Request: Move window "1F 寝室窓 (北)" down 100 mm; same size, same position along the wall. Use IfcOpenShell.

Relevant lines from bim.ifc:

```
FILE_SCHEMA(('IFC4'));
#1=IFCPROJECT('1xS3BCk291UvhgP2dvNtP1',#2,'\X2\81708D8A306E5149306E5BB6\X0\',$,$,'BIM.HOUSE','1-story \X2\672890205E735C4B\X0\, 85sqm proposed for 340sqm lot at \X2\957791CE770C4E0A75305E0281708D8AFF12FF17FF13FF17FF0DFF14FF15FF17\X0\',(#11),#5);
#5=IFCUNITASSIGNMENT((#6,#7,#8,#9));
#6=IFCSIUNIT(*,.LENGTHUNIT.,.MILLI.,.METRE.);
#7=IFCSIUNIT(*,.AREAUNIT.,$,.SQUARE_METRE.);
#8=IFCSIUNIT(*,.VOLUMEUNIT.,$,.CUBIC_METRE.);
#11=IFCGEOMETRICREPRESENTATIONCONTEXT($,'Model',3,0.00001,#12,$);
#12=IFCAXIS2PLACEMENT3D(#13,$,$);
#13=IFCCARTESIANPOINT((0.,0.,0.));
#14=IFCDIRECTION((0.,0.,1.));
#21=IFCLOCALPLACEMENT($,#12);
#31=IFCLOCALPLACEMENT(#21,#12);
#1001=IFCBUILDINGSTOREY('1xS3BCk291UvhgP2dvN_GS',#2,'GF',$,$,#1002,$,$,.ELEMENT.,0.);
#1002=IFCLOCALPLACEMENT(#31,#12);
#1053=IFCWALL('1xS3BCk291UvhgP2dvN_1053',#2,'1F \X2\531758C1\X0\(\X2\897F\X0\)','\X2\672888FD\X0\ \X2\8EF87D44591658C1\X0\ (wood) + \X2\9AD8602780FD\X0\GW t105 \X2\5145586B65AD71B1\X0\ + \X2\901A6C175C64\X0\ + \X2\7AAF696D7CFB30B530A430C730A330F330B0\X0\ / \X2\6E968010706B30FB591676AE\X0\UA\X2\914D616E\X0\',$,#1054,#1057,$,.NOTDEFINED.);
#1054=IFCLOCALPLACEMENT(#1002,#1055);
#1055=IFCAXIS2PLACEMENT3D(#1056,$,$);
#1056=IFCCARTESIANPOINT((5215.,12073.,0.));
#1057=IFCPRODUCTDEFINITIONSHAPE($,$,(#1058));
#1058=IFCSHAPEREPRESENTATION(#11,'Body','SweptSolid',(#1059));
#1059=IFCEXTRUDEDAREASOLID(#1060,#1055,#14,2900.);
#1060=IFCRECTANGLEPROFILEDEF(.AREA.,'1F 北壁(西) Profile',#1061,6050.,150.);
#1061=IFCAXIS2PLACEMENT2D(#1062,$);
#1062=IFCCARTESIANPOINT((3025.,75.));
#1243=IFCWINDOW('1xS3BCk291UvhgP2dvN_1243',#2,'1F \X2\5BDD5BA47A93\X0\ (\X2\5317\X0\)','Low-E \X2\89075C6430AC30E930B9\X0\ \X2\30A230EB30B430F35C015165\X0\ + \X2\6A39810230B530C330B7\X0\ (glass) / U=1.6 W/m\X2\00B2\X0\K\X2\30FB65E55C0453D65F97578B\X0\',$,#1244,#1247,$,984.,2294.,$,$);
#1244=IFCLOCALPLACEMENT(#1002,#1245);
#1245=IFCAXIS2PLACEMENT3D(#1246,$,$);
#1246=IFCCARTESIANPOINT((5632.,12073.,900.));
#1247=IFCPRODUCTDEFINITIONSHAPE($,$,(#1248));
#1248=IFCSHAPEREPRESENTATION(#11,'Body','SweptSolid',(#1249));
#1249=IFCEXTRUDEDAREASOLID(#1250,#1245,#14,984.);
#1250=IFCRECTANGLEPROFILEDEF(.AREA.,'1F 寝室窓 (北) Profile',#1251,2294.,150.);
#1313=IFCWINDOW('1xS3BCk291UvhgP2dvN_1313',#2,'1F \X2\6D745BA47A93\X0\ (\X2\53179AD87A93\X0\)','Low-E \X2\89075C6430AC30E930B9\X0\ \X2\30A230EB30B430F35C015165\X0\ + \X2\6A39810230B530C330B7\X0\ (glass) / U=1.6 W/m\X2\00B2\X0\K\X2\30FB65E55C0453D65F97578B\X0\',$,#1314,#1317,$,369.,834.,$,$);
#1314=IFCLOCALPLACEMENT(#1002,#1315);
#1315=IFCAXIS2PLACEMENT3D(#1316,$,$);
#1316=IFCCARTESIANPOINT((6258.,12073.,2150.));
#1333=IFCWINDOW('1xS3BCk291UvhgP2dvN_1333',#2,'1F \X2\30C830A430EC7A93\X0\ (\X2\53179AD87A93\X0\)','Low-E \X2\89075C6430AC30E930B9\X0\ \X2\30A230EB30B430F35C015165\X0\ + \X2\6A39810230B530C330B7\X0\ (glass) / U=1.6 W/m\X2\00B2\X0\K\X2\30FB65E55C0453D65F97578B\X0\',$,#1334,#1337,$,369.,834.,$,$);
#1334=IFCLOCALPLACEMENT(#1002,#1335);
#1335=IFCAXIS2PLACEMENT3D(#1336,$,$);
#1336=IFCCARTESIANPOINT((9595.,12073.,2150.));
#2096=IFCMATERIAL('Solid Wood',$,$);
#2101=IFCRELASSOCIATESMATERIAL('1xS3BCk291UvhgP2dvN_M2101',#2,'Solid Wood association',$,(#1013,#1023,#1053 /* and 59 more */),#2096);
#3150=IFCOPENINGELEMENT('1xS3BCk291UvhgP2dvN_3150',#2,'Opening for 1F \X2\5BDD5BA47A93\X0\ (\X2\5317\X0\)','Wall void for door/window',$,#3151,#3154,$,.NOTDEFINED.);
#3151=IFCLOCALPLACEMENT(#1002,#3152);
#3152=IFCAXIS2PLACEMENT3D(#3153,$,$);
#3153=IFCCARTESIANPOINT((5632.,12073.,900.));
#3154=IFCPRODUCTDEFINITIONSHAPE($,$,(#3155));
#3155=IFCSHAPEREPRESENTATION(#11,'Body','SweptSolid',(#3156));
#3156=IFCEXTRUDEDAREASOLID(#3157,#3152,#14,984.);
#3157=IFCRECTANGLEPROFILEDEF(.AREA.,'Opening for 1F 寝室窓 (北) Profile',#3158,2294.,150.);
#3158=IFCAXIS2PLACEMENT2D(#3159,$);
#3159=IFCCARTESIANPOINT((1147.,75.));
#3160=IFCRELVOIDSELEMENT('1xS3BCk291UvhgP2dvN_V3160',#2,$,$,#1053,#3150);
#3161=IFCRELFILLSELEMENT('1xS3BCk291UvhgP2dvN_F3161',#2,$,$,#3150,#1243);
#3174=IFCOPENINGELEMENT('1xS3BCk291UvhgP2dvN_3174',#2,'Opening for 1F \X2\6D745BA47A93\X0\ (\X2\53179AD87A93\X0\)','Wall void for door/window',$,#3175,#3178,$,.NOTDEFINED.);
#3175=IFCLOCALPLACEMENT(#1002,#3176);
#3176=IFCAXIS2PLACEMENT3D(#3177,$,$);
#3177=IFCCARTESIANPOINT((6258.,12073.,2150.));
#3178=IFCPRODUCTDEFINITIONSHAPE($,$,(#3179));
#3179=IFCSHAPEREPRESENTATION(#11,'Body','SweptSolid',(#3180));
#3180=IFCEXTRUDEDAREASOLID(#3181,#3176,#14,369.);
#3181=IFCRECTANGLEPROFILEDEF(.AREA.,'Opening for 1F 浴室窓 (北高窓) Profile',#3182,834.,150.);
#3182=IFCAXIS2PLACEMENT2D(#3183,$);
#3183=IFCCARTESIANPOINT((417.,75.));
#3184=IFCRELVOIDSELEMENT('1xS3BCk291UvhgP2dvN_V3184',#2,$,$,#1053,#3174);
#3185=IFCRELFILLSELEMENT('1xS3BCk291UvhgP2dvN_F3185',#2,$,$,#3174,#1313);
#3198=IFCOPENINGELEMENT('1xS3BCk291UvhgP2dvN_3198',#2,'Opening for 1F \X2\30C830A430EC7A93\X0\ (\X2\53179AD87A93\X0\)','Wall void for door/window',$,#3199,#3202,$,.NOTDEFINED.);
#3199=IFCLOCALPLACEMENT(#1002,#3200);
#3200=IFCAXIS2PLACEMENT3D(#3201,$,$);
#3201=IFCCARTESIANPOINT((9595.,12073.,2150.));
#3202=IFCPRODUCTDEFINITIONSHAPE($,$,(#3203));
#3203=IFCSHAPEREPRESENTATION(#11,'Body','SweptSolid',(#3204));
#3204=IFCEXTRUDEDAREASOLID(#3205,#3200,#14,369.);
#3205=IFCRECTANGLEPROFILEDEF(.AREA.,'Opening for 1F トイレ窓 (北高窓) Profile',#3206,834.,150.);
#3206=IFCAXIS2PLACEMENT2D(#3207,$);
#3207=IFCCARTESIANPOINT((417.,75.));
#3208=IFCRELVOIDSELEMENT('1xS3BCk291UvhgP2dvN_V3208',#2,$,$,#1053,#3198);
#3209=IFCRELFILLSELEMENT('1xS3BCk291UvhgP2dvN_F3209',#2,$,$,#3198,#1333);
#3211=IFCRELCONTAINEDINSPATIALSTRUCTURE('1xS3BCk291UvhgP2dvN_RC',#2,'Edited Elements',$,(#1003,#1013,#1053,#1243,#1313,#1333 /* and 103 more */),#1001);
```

```python
import numpy as np
import ifcopenshell
import ifcopenshell.api.geometry
import ifcopenshell.util.placement
import ifcopenshell.util.unit

model = ifcopenshell.open("bim.ifc")
unit_scale = ifcopenshell.util.unit.calculate_unit_scale(model)

window = model.by_guid("1xS3BCk291UvhgP2dvN_1243")
opening = window.FillsVoids[0].RelatingOpeningElement
dz = -100.0

shift = np.array([0.0, 0.0, dz])
# The window is not placed relative to its opening, so move both.
for product in (opening, window):
    matrix = ifcopenshell.util.placement.get_local_placement(product.ObjectPlacement)
    matrix[:3, 3] += shift
    ifcopenshell.api.geometry.edit_object_placement(model, product=product, matrix=matrix, is_si=False)

print(f"moved by {dz * unit_scale:+.3f} m")

model.write("bim_edited.ifc")
```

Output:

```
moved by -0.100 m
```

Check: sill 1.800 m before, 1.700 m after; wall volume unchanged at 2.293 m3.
